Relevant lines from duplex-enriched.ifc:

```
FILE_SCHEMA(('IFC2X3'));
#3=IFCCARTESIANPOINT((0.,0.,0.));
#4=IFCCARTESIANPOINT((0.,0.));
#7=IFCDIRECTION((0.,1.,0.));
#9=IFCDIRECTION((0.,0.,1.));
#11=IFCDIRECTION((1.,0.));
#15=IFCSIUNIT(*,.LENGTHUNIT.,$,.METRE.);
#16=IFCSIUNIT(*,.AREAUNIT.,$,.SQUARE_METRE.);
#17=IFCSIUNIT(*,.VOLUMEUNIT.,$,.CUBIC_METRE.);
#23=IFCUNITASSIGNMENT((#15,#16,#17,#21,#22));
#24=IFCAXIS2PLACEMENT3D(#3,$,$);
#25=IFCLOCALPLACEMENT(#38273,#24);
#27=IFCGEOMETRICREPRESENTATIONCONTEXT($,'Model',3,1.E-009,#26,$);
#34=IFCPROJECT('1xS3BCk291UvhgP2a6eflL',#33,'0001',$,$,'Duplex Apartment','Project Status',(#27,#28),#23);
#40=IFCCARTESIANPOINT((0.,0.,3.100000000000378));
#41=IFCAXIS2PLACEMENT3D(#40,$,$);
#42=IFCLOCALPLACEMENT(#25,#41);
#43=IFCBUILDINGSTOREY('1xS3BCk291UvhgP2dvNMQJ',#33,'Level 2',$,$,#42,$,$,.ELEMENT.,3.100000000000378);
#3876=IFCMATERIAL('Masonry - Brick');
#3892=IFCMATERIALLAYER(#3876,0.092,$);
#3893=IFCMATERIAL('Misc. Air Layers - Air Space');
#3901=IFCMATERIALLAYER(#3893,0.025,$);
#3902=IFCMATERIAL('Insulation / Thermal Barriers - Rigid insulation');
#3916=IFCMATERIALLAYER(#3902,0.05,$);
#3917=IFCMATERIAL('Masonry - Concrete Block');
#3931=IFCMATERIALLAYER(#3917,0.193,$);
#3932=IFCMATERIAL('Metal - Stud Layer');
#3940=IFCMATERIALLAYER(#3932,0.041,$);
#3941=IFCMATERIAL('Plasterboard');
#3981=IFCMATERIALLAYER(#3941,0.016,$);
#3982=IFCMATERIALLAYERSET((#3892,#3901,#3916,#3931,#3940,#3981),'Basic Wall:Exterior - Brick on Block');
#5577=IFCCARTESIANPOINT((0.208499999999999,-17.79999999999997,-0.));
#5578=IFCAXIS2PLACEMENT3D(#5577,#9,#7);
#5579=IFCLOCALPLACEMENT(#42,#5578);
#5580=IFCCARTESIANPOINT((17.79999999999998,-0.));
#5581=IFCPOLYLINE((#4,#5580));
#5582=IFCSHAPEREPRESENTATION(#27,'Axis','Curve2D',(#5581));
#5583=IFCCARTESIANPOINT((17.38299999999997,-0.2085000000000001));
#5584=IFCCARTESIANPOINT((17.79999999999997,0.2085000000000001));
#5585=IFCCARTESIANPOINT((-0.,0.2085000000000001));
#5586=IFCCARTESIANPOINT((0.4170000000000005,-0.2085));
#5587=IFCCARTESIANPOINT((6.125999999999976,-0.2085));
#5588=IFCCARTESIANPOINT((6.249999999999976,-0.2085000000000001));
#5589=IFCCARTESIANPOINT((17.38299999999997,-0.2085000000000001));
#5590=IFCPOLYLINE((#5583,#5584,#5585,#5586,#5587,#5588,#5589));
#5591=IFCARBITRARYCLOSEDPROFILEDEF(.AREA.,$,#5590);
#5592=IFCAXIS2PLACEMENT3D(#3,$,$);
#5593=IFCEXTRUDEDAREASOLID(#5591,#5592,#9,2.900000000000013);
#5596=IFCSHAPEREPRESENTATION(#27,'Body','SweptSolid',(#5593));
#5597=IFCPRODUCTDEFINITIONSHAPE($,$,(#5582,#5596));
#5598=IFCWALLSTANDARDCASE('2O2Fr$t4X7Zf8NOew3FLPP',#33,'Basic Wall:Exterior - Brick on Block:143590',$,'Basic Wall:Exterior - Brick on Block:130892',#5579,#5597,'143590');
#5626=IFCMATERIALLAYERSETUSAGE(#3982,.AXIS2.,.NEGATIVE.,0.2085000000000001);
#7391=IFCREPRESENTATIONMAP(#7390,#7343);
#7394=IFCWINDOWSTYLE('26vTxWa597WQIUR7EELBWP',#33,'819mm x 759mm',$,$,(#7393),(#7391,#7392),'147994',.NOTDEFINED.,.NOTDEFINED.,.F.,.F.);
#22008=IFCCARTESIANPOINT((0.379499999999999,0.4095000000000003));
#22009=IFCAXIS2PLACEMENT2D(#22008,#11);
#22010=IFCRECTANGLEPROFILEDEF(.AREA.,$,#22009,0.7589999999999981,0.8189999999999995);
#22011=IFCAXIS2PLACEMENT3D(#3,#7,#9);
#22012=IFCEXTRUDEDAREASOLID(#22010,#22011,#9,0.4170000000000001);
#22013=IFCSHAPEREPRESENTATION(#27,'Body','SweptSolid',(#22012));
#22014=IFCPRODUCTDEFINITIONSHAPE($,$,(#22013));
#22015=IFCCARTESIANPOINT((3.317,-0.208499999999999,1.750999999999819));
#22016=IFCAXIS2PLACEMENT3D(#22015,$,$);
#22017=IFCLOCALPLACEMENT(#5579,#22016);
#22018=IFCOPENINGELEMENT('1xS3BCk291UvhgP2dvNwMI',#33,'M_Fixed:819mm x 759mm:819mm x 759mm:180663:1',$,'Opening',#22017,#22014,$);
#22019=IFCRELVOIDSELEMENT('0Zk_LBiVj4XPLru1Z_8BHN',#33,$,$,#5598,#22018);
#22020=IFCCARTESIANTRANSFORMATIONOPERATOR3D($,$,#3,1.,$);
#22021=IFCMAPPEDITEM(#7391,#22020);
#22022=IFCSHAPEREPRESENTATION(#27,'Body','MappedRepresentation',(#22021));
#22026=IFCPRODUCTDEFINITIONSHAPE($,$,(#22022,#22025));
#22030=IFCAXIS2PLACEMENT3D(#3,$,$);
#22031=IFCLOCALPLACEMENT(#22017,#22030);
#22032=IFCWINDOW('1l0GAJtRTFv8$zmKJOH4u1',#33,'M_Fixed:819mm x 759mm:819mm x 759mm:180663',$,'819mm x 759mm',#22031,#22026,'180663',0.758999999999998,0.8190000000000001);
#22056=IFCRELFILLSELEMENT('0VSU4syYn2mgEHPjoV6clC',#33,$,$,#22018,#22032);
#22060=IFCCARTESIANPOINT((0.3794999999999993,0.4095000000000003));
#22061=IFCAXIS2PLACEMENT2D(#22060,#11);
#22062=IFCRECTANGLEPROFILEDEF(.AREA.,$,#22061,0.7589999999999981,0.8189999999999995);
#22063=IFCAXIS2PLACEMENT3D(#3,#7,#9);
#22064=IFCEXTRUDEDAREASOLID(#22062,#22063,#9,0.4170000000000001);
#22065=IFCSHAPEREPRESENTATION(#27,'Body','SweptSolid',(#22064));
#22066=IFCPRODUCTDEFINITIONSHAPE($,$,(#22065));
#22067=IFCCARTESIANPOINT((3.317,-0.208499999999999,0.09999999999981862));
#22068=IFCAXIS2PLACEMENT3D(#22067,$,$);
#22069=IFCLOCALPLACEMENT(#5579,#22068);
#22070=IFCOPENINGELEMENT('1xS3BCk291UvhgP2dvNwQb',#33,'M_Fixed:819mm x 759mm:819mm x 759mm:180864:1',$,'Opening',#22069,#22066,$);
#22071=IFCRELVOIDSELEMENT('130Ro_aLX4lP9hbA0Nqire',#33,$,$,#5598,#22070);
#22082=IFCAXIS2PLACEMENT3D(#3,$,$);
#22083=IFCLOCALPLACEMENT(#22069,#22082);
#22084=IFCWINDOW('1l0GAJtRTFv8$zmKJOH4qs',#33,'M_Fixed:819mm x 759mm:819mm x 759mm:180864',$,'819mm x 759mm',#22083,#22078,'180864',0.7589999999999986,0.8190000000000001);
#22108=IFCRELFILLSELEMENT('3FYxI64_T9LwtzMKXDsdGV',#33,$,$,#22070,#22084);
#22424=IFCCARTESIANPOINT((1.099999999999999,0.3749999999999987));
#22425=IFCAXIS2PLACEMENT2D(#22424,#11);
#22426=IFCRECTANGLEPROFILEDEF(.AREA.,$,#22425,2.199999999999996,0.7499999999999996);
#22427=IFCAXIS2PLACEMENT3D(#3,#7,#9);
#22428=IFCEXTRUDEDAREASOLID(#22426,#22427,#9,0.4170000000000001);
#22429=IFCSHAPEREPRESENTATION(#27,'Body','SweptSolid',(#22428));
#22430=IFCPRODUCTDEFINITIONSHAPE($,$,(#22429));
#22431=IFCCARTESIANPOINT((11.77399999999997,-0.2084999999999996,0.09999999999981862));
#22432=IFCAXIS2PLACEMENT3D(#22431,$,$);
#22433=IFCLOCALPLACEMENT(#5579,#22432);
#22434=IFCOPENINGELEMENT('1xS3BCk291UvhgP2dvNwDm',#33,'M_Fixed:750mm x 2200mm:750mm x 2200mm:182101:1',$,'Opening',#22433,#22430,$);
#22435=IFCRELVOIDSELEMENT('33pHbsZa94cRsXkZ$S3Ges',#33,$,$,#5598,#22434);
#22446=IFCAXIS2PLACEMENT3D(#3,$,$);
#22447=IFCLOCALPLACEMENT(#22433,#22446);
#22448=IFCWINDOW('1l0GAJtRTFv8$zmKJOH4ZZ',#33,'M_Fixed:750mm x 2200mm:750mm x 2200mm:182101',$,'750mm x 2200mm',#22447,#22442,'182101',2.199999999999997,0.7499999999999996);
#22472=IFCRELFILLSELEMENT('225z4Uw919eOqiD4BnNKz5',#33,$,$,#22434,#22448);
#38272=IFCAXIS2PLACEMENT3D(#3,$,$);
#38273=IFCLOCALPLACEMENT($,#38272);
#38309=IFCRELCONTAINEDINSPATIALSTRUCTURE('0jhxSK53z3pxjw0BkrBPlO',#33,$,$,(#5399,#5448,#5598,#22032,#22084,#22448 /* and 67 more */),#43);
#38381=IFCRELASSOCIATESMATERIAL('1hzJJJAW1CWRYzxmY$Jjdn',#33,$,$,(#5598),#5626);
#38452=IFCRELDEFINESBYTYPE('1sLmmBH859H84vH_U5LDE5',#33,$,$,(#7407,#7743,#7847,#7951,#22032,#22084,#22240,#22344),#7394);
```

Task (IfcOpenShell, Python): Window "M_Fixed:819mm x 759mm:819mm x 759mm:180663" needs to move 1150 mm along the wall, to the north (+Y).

```python
import ifcopenshell
import ifcopenshell.api.geometry
import ifcopenshell.util.placement
import ifcopenshell.util.unit

model = ifcopenshell.open("duplex-enriched.ifc")
unit_scale = ifcopenshell.util.unit.calculate_unit_scale(model)

window = model.by_guid("1l0GAJtRTFv8$zmKJOH4u1")
opening = window.FillsVoids[0].RelatingOpeningElement
wall = opening.VoidsElements[0].RelatingBuildingElement

wall_matrix = ifcopenshell.util.placement.get_local_placement(wall.ObjectPlacement)
shift = wall_matrix[:3, 0] * 1.15 / unit_scale
before = ifcopenshell.util.placement.get_local_placement(window.ObjectPlacement)[:3, 3].copy()

# The window is placed relative to its opening, so it follows when the opening moves.
matrix = ifcopenshell.util.placement.get_local_placement(opening.ObjectPlacement)
matrix[:3, 3] += shift
ifcopenshell.api.geometry.edit_object_placement(
    model, product=opening, matrix=matrix, is_si=False, should_transform_children=True
)

after = ifcopenshell.util.placement.get_local_placement(window.ObjectPlacement)[:3, 3]
print("window moved by", (after - before).round(3) + 0.0)

model.write("duplex-enriched_edited.ifc")
```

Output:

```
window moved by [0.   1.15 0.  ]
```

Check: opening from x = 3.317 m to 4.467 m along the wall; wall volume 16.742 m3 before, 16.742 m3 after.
